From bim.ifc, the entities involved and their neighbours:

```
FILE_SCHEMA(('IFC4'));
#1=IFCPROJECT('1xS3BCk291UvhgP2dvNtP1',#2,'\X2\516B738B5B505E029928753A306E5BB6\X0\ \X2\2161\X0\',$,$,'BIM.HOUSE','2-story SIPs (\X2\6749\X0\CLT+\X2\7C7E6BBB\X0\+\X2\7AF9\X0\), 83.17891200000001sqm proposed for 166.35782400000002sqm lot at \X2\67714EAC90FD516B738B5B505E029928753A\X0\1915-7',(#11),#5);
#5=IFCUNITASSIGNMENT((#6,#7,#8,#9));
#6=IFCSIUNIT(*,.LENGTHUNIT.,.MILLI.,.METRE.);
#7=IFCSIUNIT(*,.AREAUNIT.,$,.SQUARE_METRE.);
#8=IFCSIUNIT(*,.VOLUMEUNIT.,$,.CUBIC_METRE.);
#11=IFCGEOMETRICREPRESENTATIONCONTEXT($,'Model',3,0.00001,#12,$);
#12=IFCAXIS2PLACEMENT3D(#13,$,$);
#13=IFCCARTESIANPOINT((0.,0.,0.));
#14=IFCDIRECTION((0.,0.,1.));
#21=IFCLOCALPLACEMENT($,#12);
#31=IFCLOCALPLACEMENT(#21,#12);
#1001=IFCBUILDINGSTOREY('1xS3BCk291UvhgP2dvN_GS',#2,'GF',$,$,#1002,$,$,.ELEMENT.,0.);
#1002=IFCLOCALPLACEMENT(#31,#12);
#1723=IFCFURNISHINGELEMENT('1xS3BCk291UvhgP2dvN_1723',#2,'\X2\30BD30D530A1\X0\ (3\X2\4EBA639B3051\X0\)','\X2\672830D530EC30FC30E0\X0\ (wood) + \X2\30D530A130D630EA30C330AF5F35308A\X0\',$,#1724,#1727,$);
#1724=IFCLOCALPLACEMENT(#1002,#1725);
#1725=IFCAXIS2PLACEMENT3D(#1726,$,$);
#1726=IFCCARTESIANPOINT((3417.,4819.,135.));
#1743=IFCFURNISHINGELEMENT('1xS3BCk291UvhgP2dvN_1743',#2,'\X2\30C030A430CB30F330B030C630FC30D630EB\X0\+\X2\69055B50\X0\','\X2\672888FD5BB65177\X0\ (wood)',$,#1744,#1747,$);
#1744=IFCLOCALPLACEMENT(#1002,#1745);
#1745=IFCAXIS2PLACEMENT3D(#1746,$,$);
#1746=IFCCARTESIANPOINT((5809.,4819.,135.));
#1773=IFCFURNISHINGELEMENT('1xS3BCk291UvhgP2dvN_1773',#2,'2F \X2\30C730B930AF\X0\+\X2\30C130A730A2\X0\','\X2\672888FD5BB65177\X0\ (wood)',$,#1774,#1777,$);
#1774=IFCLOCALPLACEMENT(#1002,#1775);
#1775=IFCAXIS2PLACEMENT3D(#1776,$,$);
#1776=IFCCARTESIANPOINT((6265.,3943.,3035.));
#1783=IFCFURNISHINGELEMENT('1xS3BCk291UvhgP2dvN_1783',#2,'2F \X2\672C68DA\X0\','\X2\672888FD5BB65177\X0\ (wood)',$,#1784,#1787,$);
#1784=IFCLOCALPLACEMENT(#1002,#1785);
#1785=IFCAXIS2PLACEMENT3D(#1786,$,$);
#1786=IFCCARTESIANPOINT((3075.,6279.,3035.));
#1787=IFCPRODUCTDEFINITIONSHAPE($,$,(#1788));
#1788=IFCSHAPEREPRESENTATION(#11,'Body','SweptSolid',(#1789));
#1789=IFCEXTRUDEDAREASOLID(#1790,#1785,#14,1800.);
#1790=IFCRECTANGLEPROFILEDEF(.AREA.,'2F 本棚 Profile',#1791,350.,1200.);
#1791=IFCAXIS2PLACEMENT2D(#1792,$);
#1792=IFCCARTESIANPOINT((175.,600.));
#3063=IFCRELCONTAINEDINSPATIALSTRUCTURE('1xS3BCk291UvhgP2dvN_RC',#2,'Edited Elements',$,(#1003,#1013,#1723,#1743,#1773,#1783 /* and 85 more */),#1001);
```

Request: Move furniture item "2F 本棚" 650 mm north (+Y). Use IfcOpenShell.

```python
import ifcopenshell
import ifcopenshell.api.geometry
import ifcopenshell.util.placement
import ifcopenshell.util.unit

model = ifcopenshell.open("bim.ifc")
unit_scale = ifcopenshell.util.unit.calculate_unit_scale(model)

item = model.by_guid("1xS3BCk291UvhgP2dvN_1783")
matrix = ifcopenshell.util.placement.get_local_placement(item.ObjectPlacement)
matrix[1, 3] += 0.65 / unit_scale
ifcopenshell.api.geometry.edit_object_placement(model, product=item, matrix=matrix, is_si=False)

print(ifcopenshell.util.placement.get_local_placement(item.ObjectPlacement).round(3) + 0.0)

model.write("bim_edited.ifc")
```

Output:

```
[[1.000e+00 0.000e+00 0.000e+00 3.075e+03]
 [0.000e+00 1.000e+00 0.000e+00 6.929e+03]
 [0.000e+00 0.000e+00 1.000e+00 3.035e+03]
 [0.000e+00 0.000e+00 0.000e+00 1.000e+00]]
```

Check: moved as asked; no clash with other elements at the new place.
